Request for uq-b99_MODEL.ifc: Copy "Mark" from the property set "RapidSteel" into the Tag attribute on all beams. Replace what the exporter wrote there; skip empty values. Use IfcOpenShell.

First a look at what the model holds.

```python
import ifcopenshell
import ifcopenshell.util.element

model = ifcopenshell.open("uq-b99_MODEL.ifc")
print(model.schema)
beams = model.by_type("IfcBeam")
print(len(beams), "beams")
for e in beams[:8]:
    source = ifcopenshell.util.element.get_pset(e, "RapidSteel", "Mark")
    target = e.Tag
    print(e.id(), repr(source), repr(target), sep=" | ")
```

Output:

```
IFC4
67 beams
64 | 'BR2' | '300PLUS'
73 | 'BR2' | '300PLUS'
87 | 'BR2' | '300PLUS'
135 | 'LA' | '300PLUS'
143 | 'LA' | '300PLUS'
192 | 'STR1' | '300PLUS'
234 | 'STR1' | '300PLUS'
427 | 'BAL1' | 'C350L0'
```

```python
import ifcopenshell
import ifcopenshell.util.element

model = ifcopenshell.open("uq-b99_MODEL.ifc")

count = 0
for e in model.by_type("IfcBeam"):
    value = ifcopenshell.util.element.get_pset(e, "RapidSteel", "Mark")
    current = e.Tag
    if not value or not value.strip() or current == value:
        continue
    e.Tag = value
    count += 1

print(count, "beams updated")

model.write("uq-b99_MODEL_updated.ifc")
```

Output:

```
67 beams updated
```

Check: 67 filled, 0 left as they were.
